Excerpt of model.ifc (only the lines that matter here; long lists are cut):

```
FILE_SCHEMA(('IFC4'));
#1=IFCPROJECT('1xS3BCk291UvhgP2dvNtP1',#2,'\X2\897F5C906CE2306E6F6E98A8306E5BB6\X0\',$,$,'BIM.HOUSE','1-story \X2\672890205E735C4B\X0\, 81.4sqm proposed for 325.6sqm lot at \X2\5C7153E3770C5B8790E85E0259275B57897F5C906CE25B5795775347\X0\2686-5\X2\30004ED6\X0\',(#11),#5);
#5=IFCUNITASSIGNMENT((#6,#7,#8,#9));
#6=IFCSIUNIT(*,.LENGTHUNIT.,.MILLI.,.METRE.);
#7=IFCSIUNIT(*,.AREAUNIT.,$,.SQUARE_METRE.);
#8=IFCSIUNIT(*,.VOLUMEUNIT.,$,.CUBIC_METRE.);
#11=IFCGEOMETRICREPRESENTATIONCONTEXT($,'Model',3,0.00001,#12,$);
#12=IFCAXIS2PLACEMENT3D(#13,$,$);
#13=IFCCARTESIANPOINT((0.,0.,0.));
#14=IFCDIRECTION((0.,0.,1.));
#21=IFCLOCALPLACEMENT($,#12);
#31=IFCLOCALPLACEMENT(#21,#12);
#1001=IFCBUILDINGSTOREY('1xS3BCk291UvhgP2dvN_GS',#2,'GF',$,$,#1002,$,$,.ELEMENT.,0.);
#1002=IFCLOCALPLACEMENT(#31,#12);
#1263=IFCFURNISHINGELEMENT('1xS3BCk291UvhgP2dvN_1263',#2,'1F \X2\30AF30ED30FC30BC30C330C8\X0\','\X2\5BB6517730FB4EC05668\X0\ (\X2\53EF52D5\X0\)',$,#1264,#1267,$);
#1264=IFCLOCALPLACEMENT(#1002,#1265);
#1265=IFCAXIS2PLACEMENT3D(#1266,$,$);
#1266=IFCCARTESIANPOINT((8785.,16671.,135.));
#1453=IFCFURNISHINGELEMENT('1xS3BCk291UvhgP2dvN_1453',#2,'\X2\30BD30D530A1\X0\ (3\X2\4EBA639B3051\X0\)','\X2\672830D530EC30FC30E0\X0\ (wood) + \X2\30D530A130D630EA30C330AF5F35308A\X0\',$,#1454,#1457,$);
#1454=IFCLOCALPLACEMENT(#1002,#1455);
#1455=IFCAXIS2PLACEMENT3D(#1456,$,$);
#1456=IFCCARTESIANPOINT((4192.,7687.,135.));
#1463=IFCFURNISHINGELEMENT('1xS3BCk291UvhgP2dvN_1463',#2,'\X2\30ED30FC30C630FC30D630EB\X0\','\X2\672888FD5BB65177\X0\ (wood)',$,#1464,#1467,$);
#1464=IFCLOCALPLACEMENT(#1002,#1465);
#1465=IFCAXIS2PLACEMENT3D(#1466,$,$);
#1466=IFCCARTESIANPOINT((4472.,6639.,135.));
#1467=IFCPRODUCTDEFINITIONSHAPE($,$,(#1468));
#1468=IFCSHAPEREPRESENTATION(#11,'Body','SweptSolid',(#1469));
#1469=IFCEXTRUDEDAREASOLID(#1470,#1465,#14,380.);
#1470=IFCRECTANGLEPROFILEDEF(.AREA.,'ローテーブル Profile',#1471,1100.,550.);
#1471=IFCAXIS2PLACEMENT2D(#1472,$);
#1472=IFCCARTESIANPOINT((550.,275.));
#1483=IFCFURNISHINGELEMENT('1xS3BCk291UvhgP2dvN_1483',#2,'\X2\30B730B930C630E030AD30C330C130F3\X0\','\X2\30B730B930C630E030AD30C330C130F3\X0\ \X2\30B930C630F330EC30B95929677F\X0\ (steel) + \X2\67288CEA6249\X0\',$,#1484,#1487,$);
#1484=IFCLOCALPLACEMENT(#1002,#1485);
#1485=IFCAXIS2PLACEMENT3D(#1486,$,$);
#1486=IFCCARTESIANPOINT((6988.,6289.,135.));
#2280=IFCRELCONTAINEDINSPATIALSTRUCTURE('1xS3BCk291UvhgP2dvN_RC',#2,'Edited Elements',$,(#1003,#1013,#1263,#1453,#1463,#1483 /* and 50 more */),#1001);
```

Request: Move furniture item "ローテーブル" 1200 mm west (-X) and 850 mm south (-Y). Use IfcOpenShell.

```python
import ifcopenshell
import ifcopenshell.api.geometry
import ifcopenshell.util.placement
import ifcopenshell.util.unit

model = ifcopenshell.open("model.ifc")
unit_scale = ifcopenshell.util.unit.calculate_unit_scale(model)

item = model.by_guid("1xS3BCk291UvhgP2dvN_1463")
matrix = ifcopenshell.util.placement.get_local_placement(item.ObjectPlacement)
matrix[0, 3] -= 1.2 / unit_scale
matrix[1, 3] -= 0.85 / unit_scale
ifcopenshell.api.geometry.edit_object_placement(model, product=item, matrix=matrix, is_si=False)

print(ifcopenshell.util.placement.get_local_placement(item.ObjectPlacement).round(3) + 0.0)

model.write("model_edited.ifc")
```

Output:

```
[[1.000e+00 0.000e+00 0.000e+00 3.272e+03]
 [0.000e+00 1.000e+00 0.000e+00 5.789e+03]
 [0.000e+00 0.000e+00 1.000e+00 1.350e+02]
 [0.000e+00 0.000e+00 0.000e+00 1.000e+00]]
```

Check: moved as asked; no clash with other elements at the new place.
